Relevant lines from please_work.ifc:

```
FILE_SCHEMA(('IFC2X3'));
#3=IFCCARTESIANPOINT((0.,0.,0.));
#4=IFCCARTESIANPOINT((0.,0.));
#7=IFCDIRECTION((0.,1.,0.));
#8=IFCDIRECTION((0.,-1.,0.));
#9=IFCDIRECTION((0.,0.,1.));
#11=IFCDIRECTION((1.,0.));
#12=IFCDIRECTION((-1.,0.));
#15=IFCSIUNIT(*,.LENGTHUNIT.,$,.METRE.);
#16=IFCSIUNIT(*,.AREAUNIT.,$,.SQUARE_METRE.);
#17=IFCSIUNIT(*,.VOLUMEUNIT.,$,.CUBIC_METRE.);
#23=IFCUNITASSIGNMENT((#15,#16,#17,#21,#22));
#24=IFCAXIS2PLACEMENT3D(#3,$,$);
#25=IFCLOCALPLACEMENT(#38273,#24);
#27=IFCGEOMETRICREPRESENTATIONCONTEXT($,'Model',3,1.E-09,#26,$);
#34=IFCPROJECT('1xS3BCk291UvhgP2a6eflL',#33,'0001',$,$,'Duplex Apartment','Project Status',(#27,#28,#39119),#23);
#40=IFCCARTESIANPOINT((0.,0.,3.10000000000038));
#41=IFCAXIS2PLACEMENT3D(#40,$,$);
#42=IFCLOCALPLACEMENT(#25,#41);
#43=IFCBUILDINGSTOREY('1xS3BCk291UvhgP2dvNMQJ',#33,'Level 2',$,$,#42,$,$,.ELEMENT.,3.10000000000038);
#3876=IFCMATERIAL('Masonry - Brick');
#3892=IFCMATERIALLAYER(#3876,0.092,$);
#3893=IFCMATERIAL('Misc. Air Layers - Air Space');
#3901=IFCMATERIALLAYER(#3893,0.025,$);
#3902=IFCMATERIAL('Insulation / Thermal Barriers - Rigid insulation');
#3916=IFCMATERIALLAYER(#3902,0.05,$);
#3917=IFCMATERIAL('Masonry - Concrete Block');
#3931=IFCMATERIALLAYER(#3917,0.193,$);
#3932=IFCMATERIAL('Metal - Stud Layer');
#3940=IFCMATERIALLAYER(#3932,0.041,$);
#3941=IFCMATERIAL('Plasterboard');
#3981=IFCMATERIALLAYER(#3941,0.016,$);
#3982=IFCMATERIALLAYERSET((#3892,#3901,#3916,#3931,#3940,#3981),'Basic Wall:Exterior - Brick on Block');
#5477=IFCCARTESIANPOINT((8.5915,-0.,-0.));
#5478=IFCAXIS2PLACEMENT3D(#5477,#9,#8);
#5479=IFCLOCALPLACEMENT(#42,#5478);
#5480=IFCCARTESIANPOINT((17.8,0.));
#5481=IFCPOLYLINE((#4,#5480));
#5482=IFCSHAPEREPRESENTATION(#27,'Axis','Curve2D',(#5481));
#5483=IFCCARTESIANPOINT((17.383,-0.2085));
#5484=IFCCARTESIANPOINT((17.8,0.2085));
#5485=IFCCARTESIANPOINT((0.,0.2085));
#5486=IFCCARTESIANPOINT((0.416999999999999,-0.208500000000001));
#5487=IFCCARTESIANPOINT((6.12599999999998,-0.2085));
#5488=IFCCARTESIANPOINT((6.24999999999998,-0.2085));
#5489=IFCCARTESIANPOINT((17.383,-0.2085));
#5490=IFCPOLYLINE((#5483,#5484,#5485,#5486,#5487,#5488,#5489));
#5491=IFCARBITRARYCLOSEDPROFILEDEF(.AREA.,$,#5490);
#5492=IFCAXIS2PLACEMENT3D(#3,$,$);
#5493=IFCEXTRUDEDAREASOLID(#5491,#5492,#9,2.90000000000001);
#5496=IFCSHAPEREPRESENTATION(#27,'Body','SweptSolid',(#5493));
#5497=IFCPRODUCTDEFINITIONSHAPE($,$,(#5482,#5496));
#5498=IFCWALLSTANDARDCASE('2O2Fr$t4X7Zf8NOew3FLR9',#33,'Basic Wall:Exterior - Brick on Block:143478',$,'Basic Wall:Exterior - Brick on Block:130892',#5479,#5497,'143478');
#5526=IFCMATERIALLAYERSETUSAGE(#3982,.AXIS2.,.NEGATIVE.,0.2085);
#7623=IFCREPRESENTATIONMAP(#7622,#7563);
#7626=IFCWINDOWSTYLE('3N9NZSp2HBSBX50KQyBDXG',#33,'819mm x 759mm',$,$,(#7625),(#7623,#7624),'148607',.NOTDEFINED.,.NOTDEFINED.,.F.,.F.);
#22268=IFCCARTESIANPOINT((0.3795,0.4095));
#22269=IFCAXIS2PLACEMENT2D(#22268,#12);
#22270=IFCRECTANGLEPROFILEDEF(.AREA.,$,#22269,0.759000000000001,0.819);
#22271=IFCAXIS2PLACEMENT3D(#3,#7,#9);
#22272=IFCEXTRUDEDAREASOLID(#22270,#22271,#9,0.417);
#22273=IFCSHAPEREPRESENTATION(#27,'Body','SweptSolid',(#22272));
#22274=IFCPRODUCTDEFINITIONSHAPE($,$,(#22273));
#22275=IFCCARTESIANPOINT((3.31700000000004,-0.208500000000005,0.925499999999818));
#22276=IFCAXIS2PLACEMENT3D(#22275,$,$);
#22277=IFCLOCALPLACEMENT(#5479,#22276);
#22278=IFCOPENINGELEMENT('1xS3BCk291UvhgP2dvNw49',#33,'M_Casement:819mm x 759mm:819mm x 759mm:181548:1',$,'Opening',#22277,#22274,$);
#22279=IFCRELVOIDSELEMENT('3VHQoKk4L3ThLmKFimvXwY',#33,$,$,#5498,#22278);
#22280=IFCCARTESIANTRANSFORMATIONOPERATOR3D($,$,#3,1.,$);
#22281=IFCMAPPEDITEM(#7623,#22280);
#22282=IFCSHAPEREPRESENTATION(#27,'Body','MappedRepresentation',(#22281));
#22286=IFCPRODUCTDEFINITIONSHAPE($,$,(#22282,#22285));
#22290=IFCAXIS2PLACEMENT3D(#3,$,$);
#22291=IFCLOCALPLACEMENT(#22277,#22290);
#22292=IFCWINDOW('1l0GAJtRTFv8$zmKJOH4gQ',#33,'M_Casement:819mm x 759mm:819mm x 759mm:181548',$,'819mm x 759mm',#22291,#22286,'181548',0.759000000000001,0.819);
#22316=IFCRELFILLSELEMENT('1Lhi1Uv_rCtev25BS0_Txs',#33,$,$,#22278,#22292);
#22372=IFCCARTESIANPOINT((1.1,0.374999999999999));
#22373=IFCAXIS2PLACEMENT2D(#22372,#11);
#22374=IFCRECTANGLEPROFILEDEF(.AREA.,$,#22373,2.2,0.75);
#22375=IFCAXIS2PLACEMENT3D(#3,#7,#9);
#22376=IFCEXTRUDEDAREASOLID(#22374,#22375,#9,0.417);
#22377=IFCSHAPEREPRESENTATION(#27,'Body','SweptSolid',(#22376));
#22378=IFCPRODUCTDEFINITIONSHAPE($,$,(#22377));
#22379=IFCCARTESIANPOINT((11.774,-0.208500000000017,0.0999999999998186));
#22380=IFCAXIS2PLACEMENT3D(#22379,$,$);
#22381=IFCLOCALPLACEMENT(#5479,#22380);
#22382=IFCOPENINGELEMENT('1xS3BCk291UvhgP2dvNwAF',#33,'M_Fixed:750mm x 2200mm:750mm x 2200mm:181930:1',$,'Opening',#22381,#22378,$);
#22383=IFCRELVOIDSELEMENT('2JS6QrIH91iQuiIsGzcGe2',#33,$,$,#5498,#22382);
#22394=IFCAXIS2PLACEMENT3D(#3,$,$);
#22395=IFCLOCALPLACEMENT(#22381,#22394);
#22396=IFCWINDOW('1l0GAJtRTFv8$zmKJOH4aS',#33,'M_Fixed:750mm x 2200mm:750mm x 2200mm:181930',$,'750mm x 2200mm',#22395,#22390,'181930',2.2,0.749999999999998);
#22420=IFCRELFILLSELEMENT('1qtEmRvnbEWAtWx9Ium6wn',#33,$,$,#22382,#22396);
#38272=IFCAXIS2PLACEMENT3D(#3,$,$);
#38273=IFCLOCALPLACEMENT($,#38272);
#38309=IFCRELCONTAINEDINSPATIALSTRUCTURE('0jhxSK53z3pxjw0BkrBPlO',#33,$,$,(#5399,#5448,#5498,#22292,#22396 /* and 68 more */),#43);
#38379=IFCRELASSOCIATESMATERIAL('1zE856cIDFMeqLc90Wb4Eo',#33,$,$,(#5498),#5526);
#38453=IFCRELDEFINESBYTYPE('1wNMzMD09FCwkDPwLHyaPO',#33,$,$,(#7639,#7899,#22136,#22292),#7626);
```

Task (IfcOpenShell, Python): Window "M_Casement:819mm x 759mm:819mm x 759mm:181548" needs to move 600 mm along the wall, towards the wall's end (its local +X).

```python
import ifcopenshell
import ifcopenshell.api.geometry
import ifcopenshell.util.placement

model = ifcopenshell.open("please_work.ifc")

window = model.by_guid("1l0GAJtRTFv8$zmKJOH4gQ")
opening = window.FillsVoids[0].RelatingOpeningElement
wall = opening.VoidsElements[0].RelatingBuildingElement

wall_matrix = ifcopenshell.util.placement.get_local_placement(wall.ObjectPlacement)
shift = wall_matrix[:3, 0] * 0.6
before = ifcopenshell.util.placement.get_local_placement(window.ObjectPlacement)[:3, 3].copy()

# The window is placed relative to its opening, so it follows when the opening moves.
matrix = ifcopenshell.util.placement.get_local_placement(opening.ObjectPlacement)
matrix[:3, 3] += shift
ifcopenshell.api.geometry.edit_object_placement(
    model, product=opening, matrix=matrix, is_si=False, should_transform_children=True
)

after = ifcopenshell.util.placement.get_local_placement(window.ObjectPlacement)[:3, 3]
print("window moved by", (after - before).round(3) + 0.0)

model.write("please_work-out.ifc")
```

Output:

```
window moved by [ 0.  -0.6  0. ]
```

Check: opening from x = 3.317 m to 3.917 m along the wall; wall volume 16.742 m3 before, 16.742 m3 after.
